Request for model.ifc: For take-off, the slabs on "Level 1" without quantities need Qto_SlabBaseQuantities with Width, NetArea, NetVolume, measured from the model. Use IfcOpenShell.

First a look at what the model holds.

```python
import ifcopenshell
import ifcopenshell.util.element
import ifcopenshell.util.unit

model = ifcopenshell.open("model.ifc")
print(model.schema)
for unit_type in ("LENGTHUNIT", "AREAUNIT", "VOLUMEUNIT"):
    print(unit_type, ifcopenshell.util.unit.calculate_unit_scale(model, unit_type))
storey = next(s for s in model.by_type("IfcBuildingStorey") if s.Name == "Level 1")
slabs = [e for e in ifcopenshell.util.element.get_decomposition(storey) if e.is_a("IfcSlab")]
for e in sorted(slabs, key=lambda e: e.id()):
    print(e.id(), e.is_a(), e.Name, list(ifcopenshell.util.element.get_psets(e, qtos_only=True)), sep=" | ")
```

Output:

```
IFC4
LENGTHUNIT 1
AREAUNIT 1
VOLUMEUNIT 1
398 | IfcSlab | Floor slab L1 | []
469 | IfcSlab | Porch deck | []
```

```python
import ifcopenshell
import ifcopenshell.api.pset
import ifcopenshell.geom
import ifcopenshell.util.element
import ifcopenshell.util.shape
import ifcopenshell.util.unit

model = ifcopenshell.open("model.ifc")
unit_scale = ifcopenshell.util.unit.calculate_unit_scale(model)
area_scale = ifcopenshell.util.unit.calculate_unit_scale(model, "AREAUNIT")
volume_scale = ifcopenshell.util.unit.calculate_unit_scale(model, "VOLUMEUNIT")
settings = ifcopenshell.geom.settings()

storey = next(s for s in model.by_type("IfcBuildingStorey") if s.Name == "Level 1")
slabs = [e for e in ifcopenshell.util.element.get_decomposition(storey) if e.is_a("IfcSlab")]

for e in sorted(slabs, key=lambda e: e.id()):
    if ifcopenshell.util.element.get_psets(e, qtos_only=True, should_inherit=False):
        continue
    # Geometry comes back in metres, in the element's own axes.
    shape = ifcopenshell.geom.create_shape(settings, e)
    values = {
        "Width": ifcopenshell.util.shape.get_z(shape.geometry) / unit_scale,
        "NetArea": ifcopenshell.util.shape.get_footprint_area(shape.geometry) / area_scale,
        "NetVolume": ifcopenshell.util.shape.get_volume(shape.geometry) / volume_scale,
    }
    qto = ifcopenshell.api.pset.add_qto(model, product=e, name="Qto_SlabBaseQuantities")
    ifcopenshell.api.pset.edit_qto(model, qto=qto, properties=values)
    print(e.id(), {k: round(v, 3) for k, v in values.items()})

model.write("model_updated.ifc")
```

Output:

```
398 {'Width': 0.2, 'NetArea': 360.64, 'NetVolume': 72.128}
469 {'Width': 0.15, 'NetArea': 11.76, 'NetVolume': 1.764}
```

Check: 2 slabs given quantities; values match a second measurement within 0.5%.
